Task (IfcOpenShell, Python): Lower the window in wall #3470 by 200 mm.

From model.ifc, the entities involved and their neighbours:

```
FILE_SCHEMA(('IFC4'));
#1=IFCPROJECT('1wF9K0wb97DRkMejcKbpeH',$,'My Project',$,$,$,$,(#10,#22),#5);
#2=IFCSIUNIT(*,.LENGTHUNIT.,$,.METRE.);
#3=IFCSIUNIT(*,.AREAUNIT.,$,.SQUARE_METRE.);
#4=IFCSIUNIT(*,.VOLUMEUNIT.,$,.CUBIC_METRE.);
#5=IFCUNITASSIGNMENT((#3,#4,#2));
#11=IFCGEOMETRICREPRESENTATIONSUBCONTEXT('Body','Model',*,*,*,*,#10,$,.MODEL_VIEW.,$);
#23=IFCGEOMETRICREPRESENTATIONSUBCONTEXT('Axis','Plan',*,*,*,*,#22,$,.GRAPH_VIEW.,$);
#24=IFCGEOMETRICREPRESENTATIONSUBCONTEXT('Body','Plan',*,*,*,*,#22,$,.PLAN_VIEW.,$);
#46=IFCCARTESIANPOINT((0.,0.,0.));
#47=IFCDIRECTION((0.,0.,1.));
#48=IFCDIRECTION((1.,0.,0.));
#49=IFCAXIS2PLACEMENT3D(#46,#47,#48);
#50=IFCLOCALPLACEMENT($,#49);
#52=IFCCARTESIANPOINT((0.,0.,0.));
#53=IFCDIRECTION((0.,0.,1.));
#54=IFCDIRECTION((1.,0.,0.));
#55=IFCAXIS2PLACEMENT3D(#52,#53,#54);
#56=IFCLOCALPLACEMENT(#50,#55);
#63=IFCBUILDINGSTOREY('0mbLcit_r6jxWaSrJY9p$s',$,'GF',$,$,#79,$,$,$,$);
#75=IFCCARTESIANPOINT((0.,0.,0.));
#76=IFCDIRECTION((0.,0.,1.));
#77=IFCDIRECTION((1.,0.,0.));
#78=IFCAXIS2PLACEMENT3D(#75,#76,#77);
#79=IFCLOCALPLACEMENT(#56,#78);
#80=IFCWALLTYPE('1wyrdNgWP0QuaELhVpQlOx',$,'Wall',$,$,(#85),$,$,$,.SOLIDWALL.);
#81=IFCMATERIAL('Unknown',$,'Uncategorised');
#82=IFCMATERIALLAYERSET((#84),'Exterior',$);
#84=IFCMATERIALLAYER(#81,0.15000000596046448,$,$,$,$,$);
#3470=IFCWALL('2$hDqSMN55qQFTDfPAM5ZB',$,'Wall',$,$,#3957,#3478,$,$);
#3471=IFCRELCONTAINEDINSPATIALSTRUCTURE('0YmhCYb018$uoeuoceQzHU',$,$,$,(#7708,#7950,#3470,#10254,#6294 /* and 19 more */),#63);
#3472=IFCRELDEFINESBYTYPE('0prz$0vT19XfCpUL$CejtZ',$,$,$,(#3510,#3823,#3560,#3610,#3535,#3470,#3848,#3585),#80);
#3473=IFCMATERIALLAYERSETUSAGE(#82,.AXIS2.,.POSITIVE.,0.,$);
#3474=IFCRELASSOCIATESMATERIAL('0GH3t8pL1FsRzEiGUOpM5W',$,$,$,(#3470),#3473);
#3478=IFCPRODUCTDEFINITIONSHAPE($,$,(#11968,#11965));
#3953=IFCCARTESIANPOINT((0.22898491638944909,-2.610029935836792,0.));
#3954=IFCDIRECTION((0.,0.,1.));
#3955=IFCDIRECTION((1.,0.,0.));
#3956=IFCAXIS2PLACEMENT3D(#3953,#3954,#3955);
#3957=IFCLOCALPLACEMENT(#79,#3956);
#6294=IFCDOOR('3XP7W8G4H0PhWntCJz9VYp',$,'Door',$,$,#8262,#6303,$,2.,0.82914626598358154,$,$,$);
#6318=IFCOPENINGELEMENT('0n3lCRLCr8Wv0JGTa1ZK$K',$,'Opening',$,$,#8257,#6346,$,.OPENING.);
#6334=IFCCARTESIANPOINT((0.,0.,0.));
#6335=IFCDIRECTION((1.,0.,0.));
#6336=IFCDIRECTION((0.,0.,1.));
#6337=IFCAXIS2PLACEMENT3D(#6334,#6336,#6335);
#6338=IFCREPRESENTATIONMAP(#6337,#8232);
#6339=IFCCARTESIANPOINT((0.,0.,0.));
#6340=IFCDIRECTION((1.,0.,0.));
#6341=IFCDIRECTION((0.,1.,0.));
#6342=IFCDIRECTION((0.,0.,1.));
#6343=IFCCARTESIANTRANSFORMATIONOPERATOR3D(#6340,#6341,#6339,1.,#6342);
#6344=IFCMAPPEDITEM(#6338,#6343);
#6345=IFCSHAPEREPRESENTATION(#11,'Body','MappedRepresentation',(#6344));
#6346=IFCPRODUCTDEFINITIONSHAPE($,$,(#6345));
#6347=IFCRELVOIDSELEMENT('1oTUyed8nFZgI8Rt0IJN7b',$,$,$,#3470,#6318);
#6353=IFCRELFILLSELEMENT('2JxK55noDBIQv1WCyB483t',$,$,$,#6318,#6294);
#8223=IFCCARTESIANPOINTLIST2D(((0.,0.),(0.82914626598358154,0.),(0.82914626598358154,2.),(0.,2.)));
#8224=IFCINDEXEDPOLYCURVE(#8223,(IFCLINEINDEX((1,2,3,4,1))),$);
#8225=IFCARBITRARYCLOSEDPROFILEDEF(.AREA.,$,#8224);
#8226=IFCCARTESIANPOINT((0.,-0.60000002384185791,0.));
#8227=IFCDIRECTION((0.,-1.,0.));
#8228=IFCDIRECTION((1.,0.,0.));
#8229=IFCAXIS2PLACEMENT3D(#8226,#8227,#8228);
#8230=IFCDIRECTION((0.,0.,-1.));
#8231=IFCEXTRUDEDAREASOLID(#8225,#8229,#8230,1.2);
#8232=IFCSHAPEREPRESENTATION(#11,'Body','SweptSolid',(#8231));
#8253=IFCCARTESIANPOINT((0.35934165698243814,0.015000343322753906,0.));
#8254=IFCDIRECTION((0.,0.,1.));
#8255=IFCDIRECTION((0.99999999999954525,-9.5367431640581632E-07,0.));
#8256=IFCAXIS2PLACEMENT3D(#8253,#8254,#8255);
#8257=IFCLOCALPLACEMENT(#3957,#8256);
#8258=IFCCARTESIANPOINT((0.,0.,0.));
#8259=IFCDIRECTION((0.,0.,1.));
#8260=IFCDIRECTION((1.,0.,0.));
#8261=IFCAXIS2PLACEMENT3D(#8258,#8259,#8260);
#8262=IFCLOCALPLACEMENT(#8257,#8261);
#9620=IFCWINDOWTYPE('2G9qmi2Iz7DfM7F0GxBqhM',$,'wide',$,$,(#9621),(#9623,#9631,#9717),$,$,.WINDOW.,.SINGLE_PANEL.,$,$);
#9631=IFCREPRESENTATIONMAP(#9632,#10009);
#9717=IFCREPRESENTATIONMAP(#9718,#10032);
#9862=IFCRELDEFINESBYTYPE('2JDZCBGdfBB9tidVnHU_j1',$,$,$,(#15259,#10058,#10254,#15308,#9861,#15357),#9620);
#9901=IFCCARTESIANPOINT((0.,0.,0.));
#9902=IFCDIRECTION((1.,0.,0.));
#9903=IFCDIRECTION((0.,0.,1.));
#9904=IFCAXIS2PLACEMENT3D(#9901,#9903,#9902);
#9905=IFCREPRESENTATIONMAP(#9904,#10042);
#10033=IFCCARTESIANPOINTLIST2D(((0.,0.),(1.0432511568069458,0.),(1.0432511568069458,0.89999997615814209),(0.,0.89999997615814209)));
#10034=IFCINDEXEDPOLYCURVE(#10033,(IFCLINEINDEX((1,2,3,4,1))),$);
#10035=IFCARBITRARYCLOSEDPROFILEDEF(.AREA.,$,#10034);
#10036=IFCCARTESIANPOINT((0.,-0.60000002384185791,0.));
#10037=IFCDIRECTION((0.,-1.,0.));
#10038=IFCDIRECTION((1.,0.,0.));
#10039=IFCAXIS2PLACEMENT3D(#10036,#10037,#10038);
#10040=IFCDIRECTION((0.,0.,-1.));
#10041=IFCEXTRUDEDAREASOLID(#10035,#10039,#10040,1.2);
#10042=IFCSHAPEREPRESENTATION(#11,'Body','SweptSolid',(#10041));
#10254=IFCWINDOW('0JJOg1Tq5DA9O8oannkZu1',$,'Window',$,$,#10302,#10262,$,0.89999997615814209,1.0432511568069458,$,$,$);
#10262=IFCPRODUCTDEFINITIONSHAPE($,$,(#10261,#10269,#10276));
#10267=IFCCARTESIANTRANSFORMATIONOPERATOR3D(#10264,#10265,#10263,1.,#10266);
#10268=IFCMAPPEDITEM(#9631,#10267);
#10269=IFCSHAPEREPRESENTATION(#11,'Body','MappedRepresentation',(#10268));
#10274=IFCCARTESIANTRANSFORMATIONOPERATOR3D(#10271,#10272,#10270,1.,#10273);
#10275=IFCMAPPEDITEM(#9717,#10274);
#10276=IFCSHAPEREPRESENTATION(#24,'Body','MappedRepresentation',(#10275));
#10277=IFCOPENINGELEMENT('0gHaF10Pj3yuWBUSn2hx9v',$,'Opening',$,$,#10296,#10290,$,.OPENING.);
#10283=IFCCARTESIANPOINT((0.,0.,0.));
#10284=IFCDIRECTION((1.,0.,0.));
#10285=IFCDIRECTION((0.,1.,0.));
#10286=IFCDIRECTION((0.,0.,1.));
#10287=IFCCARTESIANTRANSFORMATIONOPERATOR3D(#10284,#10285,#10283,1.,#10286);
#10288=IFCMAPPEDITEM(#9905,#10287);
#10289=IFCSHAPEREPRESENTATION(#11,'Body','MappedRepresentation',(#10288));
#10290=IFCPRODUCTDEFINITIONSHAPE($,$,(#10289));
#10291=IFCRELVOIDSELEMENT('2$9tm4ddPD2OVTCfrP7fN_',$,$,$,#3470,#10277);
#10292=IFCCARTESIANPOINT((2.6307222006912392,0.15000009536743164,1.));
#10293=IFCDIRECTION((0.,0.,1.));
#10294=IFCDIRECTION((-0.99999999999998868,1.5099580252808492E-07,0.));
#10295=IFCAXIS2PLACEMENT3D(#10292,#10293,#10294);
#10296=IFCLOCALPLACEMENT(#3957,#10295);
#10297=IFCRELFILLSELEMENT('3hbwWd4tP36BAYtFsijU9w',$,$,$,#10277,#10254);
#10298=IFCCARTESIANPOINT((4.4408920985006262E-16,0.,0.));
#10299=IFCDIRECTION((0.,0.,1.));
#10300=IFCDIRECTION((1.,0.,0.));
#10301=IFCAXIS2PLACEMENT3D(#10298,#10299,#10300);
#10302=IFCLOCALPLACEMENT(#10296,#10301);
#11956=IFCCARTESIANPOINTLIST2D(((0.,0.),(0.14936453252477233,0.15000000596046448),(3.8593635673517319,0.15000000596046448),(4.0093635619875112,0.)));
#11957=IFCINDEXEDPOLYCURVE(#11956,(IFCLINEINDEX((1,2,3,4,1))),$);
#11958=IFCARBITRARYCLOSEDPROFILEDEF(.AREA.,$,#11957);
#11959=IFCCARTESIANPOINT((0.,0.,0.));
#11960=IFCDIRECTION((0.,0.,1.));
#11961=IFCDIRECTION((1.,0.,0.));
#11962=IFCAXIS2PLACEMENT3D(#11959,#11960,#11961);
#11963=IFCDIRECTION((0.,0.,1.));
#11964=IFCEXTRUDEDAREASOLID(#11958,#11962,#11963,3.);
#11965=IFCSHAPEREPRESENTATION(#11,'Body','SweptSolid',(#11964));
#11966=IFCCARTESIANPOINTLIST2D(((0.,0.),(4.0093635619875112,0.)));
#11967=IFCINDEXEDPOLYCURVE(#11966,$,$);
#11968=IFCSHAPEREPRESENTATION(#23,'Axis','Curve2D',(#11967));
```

```python
import numpy as np
import ifcopenshell
import ifcopenshell.api.geometry
import ifcopenshell.util.placement
import ifcopenshell.util.unit

model = ifcopenshell.open("model.ifc")
unit_scale = ifcopenshell.util.unit.calculate_unit_scale(model)

window = model.by_guid("0JJOg1Tq5DA9O8oannkZu1")
opening = window.FillsVoids[0].RelatingOpeningElement
dz = -0.2 / unit_scale

shift = np.array([0.0, 0.0, dz])
# The window is placed relative to its opening, so it follows when the opening moves.
matrix = ifcopenshell.util.placement.get_local_placement(opening.ObjectPlacement)
matrix[:3, 3] += shift
ifcopenshell.api.geometry.edit_object_placement(
    model, product=opening, matrix=matrix, is_si=False, should_transform_children=True
)

print(f"moved by {dz * unit_scale:+.3f} m")

model.write("model_updated.ifc")
```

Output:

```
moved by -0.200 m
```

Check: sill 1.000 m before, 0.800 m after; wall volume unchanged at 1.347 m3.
